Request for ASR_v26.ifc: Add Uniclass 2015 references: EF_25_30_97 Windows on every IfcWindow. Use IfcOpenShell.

First a look at what the model holds.

```python
import ifcopenshell

model = ifcopenshell.open("ASR_v26.ifc")
print(model.schema)
print("classifications:", [c.Name for c in model.by_type("IfcClassification")])
for ifc_class in ("IfcDoor", "IfcRoof", "IfcStair", "IfcWall", "IfcWindow"):
    print(ifc_class, len(model.by_type(ifc_class)))
```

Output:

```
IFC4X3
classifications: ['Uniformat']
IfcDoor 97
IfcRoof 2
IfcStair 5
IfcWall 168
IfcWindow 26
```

```python
import ifcopenshell
import ifcopenshell.api.classification

model = ifcopenshell.open("ASR_v26.ifc")

system = ifcopenshell.api.classification.add_classification(model, classification="Uniclass 2015")

codes = {
    "IfcWindow": ("EF_25_30_97", "Windows"),
}
for ifc_class, (code, name) in codes.items():
    products = model.by_type(ifc_class)
    ifcopenshell.api.classification.add_reference(
        model, products=products, classification=system, identification=code, name=name
    )
    print(code, len(products))

model.write("ASR_v26_v2.ifc")
```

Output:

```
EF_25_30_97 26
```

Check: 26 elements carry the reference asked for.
